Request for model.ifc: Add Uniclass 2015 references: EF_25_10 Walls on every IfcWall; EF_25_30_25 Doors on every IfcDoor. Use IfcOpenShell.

First a look at what the model holds.

```python
import ifcopenshell

model = ifcopenshell.open("model.ifc")
print(model.schema)
print("classifications:", [c.Name for c in model.by_type("IfcClassification")])
for ifc_class in ("IfcDoor", "IfcRoof", "IfcStair", "IfcWall", "IfcWindow"):
    print(ifc_class, len(model.by_type(ifc_class)))
```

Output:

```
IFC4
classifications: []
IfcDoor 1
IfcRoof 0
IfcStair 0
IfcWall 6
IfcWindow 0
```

```python
import ifcopenshell
import ifcopenshell.api.classification

model = ifcopenshell.open("model.ifc")

system = ifcopenshell.api.classification.add_classification(model, classification="Uniclass 2015")

codes = {
    "IfcWall": ("EF_25_10", "Walls"),
    "IfcDoor": ("EF_25_30_25", "Doors"),
}
for ifc_class, (code, name) in codes.items():
    products = model.by_type(ifc_class)
    ifcopenshell.api.classification.add_reference(
        model, products=products, classification=system, identification=code, name=name
    )
    print(code, len(products))

model.write("model-out.ifc")
```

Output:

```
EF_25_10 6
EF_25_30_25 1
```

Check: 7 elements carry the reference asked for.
